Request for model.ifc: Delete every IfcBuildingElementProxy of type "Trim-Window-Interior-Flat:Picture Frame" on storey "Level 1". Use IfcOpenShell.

First a look at what the model holds.

```python
import ifcopenshell
import ifcopenshell.util.element

model = ifcopenshell.open("model.ifc")
print(model.schema)
storey = next(s for s in model.by_type("IfcBuildingStorey") if s.Name == "Level 1")
proxies = [e for e in ifcopenshell.util.element.get_decomposition(storey) if e.is_a("IfcBuildingElementProxy")]
seen = {}
for e in proxies:
    element_type = ifcopenshell.util.element.get_type(e)
    name = element_type.Name if element_type not in (None, e) else None
    seen[name] = seen.get(name, 0) + 1
for name, count in sorted(seen.items(), key=str):
    print(count, "x", name)
```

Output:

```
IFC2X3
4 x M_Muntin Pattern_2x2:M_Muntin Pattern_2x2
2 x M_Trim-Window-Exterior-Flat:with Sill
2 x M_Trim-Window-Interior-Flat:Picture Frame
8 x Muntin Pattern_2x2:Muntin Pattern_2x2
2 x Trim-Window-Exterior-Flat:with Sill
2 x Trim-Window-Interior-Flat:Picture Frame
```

```python
import ifcopenshell
import ifcopenshell.api.root
import ifcopenshell.util.element

model = ifcopenshell.open("model.ifc")

storey = next(s for s in model.by_type("IfcBuildingStorey") if s.Name == "Level 1")
proxies = [e for e in ifcopenshell.util.element.get_decomposition(storey) if e.is_a("IfcBuildingElementProxy")]
targets = [e for e in proxies if (t := ifcopenshell.util.element.get_type(e)) not in (None, e) and t.Name == "Trim-Window-Interior-Flat:Picture Frame"]

for e in targets:
    ifcopenshell.api.root.remove_product(model, product=e)
print(len(targets), "removed")

model.write("model_updated.ifc")
```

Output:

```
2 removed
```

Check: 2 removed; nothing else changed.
